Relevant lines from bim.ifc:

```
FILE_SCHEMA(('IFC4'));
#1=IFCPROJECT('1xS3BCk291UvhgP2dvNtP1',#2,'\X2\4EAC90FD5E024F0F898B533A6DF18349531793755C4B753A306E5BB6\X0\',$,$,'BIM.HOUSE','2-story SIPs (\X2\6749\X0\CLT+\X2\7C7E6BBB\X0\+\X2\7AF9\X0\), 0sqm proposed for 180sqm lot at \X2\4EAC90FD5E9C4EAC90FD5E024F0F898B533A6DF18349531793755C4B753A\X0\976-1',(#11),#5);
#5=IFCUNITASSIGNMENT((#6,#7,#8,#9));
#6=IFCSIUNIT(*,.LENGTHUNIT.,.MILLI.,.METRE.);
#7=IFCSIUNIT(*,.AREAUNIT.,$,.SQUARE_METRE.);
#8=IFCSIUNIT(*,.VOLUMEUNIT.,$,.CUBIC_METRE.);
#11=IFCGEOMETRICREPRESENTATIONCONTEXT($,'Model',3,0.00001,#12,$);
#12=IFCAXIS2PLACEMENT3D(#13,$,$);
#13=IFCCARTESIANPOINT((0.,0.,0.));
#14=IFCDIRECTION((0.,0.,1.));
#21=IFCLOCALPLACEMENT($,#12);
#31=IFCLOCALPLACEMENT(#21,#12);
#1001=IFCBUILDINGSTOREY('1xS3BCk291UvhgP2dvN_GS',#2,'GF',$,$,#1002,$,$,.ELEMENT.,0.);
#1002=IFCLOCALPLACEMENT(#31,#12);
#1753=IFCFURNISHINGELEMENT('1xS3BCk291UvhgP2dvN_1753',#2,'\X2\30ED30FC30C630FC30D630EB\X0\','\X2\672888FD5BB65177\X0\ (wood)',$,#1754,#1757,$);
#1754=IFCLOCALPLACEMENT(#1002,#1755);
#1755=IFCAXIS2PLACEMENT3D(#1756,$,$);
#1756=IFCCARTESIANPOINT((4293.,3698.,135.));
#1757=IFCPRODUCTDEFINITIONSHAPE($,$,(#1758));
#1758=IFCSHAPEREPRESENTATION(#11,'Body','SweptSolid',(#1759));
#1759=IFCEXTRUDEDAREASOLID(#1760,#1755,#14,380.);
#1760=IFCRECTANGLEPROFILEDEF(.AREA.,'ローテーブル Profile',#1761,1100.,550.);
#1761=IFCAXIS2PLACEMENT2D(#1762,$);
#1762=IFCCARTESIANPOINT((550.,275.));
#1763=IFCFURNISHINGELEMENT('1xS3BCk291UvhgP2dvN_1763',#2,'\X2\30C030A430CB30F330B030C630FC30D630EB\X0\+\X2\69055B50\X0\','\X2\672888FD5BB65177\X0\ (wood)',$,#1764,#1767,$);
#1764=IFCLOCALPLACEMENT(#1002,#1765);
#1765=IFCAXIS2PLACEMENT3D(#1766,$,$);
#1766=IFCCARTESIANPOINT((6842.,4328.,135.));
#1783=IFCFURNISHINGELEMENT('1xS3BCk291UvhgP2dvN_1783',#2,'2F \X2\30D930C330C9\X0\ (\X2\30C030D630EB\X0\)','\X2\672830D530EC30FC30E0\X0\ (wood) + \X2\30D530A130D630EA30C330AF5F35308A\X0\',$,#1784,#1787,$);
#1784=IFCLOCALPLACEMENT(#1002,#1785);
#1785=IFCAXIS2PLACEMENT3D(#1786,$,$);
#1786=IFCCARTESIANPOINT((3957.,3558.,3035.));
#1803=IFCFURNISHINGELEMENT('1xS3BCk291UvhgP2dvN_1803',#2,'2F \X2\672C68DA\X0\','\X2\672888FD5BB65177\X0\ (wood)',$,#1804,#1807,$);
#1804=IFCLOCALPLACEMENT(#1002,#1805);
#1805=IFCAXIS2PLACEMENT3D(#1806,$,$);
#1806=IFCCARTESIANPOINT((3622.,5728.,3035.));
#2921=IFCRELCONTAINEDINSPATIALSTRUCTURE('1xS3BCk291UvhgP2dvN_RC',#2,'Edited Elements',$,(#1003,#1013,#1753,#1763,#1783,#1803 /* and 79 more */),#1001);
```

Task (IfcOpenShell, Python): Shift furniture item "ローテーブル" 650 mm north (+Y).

```python
import ifcopenshell
import ifcopenshell.api.geometry
import ifcopenshell.util.placement
import ifcopenshell.util.unit

model = ifcopenshell.open("bim.ifc")
unit_scale = ifcopenshell.util.unit.calculate_unit_scale(model)

item = model.by_id(1753)
matrix = ifcopenshell.util.placement.get_local_placement(item.ObjectPlacement)
matrix[1, 3] += 0.65 / unit_scale
ifcopenshell.api.geometry.edit_object_placement(model, product=item, matrix=matrix, is_si=False)

print(ifcopenshell.util.placement.get_local_placement(item.ObjectPlacement).round(3) + 0.0)

model.write("bim_edited.ifc")
```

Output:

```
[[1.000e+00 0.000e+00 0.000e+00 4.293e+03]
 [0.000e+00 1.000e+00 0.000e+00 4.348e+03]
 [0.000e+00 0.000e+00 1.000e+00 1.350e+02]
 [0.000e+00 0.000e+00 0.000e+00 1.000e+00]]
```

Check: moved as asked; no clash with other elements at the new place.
